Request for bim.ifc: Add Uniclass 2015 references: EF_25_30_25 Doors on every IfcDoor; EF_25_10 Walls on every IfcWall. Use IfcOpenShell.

First a look at what the model holds.

```python
import ifcopenshell

model = ifcopenshell.open("bim.ifc")
print(model.schema)
print("classifications:", [c.Name for c in model.by_type("IfcClassification")])
for ifc_class in ("IfcDoor", "IfcRoof", "IfcStair", "IfcWall", "IfcWindow"):
    print(ifc_class, len(model.by_type(ifc_class)))
```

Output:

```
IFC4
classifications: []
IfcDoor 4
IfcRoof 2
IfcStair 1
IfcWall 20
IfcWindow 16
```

```python
import ifcopenshell
import ifcopenshell.api.classification

model = ifcopenshell.open("bim.ifc")

system = ifcopenshell.api.classification.add_classification(model, classification="Uniclass 2015")

codes = {
    "IfcDoor": ("EF_25_30_25", "Doors"),
    "IfcWall": ("EF_25_10", "Walls"),
}
for ifc_class, (code, name) in codes.items():
    products = model.by_type(ifc_class)
    ifcopenshell.api.classification.add_reference(
        model, products=products, classification=system, identification=code, name=name
    )
    print(code, len(products))

model.write("bim-out.ifc")
```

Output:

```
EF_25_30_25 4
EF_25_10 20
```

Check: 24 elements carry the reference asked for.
